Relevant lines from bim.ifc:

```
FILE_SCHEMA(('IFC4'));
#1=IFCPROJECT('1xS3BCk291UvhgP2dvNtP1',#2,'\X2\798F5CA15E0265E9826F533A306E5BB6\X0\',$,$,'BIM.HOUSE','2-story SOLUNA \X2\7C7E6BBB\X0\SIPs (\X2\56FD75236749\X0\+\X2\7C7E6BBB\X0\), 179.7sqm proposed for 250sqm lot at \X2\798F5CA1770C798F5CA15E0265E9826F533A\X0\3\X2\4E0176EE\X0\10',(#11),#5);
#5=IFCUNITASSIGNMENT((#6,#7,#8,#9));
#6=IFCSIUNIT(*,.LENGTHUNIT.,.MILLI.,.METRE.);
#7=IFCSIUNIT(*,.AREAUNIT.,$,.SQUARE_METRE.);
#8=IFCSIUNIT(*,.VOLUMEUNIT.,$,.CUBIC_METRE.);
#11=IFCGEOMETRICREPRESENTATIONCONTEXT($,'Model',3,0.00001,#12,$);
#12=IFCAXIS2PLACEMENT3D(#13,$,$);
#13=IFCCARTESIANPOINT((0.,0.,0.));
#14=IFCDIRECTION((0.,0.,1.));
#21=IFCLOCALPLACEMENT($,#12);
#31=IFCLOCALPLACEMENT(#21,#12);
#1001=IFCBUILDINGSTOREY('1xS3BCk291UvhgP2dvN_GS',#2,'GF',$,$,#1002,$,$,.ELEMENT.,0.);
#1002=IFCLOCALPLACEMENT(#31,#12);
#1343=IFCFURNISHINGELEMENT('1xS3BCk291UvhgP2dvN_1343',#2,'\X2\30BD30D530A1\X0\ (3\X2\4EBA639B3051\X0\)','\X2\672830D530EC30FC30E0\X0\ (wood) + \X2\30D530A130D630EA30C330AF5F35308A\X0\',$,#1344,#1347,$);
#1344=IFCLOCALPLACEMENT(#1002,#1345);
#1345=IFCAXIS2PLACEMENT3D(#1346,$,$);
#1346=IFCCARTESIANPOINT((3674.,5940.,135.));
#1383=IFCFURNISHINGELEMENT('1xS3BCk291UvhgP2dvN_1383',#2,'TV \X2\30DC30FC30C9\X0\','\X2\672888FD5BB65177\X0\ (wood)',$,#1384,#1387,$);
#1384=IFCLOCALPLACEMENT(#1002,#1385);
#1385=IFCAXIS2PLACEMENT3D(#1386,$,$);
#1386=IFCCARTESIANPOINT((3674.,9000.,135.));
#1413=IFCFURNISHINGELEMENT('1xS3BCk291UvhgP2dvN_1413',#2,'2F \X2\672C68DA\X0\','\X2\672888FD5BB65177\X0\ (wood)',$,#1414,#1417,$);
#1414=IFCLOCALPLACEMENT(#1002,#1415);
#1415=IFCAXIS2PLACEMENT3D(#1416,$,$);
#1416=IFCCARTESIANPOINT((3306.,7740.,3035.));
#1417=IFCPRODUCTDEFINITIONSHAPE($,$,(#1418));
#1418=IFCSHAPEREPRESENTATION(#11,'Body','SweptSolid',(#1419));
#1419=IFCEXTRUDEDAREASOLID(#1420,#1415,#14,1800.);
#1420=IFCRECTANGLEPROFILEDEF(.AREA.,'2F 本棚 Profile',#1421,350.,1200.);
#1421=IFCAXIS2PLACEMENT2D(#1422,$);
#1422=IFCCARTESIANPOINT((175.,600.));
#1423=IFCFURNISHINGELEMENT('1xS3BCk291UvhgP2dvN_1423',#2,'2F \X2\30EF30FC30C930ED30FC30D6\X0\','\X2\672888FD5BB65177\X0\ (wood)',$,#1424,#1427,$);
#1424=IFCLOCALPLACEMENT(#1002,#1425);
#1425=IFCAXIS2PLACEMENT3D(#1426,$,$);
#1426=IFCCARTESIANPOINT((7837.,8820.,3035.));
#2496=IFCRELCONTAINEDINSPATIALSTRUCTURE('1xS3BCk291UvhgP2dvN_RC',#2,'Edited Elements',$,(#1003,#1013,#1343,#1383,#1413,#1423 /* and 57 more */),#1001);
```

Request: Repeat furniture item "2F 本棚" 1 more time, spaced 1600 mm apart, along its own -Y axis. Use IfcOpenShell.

```python
import ifcopenshell
import ifcopenshell.api.geometry
import ifcopenshell.api.root
import ifcopenshell.util.element
import ifcopenshell.util.placement
import ifcopenshell.util.unit

model = ifcopenshell.open("bim.ifc")
unit_scale = ifcopenshell.util.unit.calculate_unit_scale(model)


def reuse_history(source, copy):
    """copy_class also copies each property set's owner history, people and application; keep the originals."""
    for rel in copy.IsDefinedBy:
        if rel.is_a("IfcRelDefinesByProperties") and (history := rel.RelatingPropertyDefinition.OwnerHistory):
            rel.RelatingPropertyDefinition.OwnerHistory = source.OwnerHistory
            ifcopenshell.util.element.remove_deep2(model, history)


source = model.by_guid("1xS3BCk291UvhgP2dvN_1413")
base = ifcopenshell.util.placement.get_local_placement(source.ObjectPlacement)
step = -base[:3, 1] * 1.6 / unit_scale

for i in range(1, 2):
    copy = ifcopenshell.api.root.copy_class(model, product=source)
    copy.Representation = ifcopenshell.util.element.copy_deep(
        model, source.Representation, exclude=["IfcGeometricRepresentationContext", "IfcRepresentationMap"]
    )
    reuse_history(source, copy)
    matrix = base.copy()
    matrix[:3, 3] += i * step
    print("added at", matrix[:3, 3].round(3) + 0.0)
    ifcopenshell.api.geometry.edit_object_placement(model, product=copy, matrix=matrix, is_si=False)

model.write("bim_updated.ifc")
```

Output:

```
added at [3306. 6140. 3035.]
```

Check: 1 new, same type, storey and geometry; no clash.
